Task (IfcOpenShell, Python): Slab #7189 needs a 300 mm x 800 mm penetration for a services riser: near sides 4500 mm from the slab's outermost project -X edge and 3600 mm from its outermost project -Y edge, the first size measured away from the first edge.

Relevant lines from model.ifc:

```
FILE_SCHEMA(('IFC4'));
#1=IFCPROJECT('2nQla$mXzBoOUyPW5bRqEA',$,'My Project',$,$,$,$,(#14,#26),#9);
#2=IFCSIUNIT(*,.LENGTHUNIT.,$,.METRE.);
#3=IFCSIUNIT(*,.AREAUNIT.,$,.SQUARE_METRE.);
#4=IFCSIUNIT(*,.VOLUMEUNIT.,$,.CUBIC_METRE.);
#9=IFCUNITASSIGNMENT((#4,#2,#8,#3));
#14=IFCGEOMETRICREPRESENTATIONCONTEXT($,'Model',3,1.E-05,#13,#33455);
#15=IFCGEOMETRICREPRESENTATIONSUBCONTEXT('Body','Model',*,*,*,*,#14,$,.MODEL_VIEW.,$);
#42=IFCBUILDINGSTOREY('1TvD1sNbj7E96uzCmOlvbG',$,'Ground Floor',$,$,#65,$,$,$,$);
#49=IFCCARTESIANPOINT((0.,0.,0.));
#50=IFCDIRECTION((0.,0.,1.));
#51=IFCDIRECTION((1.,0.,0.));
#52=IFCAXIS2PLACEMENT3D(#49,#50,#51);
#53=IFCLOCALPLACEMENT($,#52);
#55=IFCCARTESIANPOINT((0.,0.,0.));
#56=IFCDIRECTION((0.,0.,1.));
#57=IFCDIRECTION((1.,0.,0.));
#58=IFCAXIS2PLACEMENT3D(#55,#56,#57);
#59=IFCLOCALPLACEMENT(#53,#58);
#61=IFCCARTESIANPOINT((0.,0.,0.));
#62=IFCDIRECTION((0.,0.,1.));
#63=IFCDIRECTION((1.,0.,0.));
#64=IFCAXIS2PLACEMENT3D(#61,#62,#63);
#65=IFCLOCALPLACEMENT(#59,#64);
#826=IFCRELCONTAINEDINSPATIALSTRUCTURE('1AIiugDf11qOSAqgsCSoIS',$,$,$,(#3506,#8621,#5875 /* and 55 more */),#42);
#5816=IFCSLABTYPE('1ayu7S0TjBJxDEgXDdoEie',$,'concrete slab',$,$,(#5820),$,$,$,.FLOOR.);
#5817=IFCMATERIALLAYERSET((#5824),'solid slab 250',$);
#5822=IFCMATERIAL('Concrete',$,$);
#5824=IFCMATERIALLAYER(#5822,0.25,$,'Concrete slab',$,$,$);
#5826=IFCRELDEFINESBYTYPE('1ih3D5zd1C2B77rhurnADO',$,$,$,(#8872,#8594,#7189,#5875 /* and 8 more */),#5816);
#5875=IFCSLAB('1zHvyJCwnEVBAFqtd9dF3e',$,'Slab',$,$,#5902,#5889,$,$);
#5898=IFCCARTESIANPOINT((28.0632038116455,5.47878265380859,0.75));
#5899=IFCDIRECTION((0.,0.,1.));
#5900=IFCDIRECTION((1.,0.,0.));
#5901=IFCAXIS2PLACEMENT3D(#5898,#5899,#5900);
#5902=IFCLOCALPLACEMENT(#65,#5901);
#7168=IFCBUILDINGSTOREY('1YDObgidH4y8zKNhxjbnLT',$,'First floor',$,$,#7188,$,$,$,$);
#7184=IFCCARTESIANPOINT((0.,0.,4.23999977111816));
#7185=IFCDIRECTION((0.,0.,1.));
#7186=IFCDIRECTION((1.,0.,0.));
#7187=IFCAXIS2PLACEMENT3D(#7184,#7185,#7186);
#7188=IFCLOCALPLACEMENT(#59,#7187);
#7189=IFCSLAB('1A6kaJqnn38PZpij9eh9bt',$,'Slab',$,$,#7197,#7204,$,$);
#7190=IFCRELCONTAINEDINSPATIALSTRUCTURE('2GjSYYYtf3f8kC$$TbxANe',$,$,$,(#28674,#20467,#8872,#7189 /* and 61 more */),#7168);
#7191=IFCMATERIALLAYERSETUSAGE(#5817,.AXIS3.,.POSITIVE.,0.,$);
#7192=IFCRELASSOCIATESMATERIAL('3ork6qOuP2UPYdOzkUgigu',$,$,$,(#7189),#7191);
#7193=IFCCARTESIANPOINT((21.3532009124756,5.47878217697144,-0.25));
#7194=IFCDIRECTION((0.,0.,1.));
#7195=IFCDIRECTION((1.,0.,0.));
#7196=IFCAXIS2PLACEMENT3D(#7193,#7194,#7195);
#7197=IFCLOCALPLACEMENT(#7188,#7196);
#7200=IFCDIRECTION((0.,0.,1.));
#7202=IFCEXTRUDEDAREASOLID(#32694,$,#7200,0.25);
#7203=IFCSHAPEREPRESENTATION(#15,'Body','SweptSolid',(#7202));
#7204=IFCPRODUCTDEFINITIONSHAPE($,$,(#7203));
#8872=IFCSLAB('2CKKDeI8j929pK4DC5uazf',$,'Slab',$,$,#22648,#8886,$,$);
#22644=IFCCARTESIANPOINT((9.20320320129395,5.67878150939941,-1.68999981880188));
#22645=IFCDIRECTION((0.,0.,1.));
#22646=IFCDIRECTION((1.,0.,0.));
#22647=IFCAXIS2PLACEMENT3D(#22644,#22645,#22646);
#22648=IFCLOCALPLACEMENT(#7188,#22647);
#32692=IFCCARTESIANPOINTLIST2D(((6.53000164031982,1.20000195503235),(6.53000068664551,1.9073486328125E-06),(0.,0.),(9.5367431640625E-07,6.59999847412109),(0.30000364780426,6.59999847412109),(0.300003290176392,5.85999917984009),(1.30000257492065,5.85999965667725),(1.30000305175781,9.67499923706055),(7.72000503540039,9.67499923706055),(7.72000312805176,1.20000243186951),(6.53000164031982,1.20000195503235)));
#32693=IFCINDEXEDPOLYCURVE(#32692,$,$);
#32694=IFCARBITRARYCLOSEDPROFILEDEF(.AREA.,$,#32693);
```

```python
import numpy as np
import ifcopenshell
import ifcopenshell.api.feature
import ifcopenshell.api.geometry
import ifcopenshell.api.root
import ifcopenshell.geom
import ifcopenshell.util.placement
import ifcopenshell.util.representation
import ifcopenshell.util.shape
import ifcopenshell.util.unit

model = ifcopenshell.open("model.ifc")
unit_scale = ifcopenshell.util.unit.calculate_unit_scale(model)
settings = ifcopenshell.geom.settings()


def volume(element):
    """Net volume in cubic metres, openings subtracted."""
    shape = ifcopenshell.geom.create_shape(settings, element)
    return ifcopenshell.util.shape.get_volume(shape.geometry)


slab = model.by_guid("1A6kaJqnn38PZpij9eh9bt")
before = volume(slab)

# Extent in the slab's own axes, in metres. The edges named are its -X and -Y sides.
slab_shape = ifcopenshell.geom.create_shape(settings, slab)
vertices = ifcopenshell.util.shape.get_vertices(slab_shape.geometry)
x_min, y_min, bottom = vertices.min(axis=0)
top = vertices[:, 2].max()

opening = ifcopenshell.api.root.create_entity(model, ifc_class="IfcOpeningElement", name="Services riser opening", predefined_type="OPENING")
context = ifcopenshell.util.representation.get_context(model, "Model", "Body", "MODEL_VIEW")
width, depth = 0.3, 0.8
outline = [(0.0, 0.0), (width, 0.0), (width, depth), (0.0, depth), (0.0, 0.0)]
# Overshoot both faces by 50 mm so the cut is clean.
shape = ifcopenshell.api.geometry.add_slab_representation(
    model, context=context, depth=top - bottom + 0.1, polyline=outline
)
ifcopenshell.api.geometry.assign_representation(model, product=opening, representation=shape)

matrix = ifcopenshell.util.placement.get_local_placement(slab.ObjectPlacement)
matrix[:, 3] = matrix @ np.append(np.array([x_min + 4.5, y_min + 3.6, bottom - 0.05]) / unit_scale, 1.0)
ifcopenshell.api.geometry.edit_object_placement(model, product=opening, matrix=matrix, is_si=False)
ifcopenshell.api.feature.add_feature(model, feature=opening, element=slab)

after = volume(slab)

print(f"slab volume {before:.3f} -> {after:.3f} m3")

model.write("model_updated.ifc")
```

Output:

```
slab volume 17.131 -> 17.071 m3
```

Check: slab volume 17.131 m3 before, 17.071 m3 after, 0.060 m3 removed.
